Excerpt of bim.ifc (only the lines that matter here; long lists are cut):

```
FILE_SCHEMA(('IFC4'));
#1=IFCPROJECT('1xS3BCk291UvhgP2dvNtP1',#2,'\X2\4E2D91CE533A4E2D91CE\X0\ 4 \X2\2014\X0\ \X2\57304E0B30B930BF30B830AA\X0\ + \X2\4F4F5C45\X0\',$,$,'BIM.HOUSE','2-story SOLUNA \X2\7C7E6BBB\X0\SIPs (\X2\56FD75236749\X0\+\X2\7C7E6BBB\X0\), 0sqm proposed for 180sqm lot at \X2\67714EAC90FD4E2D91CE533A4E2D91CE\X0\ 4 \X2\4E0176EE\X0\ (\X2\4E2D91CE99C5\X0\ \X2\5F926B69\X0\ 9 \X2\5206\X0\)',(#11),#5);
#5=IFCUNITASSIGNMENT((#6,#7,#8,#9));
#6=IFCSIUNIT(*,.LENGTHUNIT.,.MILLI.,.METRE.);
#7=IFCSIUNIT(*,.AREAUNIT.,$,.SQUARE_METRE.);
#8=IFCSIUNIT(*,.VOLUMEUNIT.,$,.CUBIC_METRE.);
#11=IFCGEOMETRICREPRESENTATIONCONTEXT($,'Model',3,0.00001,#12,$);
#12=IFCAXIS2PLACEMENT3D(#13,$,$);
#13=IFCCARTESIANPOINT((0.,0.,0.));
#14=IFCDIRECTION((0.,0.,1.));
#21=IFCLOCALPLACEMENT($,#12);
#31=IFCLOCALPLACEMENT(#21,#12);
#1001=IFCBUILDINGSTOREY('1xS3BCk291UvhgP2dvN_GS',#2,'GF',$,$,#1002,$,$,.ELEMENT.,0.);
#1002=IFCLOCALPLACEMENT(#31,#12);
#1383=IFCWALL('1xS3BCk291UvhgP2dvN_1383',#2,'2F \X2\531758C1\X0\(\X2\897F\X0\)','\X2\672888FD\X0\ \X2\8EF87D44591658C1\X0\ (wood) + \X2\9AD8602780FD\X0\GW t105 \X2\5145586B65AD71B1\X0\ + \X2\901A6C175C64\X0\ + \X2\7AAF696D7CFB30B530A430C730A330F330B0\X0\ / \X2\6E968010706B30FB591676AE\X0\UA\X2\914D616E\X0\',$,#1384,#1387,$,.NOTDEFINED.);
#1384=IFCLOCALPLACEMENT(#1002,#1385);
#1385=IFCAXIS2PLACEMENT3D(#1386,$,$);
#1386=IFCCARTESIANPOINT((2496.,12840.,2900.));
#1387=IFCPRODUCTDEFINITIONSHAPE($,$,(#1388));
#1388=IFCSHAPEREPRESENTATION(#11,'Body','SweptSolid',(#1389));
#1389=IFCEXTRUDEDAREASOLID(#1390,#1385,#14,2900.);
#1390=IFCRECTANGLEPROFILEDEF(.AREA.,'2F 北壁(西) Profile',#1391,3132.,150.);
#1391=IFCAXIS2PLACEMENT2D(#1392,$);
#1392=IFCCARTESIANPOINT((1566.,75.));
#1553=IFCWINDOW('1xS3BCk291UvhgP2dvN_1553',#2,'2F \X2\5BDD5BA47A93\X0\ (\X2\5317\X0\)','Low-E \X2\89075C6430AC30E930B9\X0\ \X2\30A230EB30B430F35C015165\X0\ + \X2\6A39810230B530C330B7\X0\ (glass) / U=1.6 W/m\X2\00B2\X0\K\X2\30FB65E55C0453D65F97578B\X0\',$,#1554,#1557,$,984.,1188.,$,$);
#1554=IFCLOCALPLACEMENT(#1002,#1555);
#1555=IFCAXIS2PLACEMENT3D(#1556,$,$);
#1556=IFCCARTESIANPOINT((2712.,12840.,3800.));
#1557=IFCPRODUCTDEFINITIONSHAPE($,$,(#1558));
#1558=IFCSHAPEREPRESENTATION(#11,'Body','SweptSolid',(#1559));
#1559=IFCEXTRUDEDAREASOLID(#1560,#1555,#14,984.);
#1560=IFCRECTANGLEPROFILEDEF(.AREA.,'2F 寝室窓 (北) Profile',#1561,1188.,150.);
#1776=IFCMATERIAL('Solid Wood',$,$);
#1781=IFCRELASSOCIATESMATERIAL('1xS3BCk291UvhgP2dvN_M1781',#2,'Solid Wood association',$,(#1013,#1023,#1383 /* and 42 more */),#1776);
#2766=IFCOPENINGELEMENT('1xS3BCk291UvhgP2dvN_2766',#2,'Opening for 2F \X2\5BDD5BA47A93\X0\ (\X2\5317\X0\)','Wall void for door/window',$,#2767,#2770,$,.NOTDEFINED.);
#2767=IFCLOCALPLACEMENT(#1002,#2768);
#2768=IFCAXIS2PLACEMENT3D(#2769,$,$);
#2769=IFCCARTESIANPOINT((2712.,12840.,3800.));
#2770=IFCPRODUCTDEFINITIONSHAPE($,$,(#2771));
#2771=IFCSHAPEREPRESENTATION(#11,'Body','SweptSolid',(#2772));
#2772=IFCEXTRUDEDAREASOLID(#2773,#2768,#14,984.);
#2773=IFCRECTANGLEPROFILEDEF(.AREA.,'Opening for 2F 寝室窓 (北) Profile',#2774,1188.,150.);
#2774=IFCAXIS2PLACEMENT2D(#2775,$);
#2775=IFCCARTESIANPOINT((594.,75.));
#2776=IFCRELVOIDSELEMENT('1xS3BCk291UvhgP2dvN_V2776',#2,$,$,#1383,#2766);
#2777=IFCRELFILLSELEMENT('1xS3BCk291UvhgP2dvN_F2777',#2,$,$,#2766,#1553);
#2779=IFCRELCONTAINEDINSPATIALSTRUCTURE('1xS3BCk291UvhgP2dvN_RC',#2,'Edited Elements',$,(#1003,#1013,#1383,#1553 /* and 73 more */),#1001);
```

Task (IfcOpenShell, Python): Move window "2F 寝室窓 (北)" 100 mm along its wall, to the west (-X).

```python
import ifcopenshell
import ifcopenshell.api.geometry
import ifcopenshell.util.placement
import ifcopenshell.util.unit

model = ifcopenshell.open("bim.ifc")
unit_scale = ifcopenshell.util.unit.calculate_unit_scale(model)

window = model.by_id(1553)
opening = window.FillsVoids[0].RelatingOpeningElement
wall = opening.VoidsElements[0].RelatingBuildingElement

wall_matrix = ifcopenshell.util.placement.get_local_placement(wall.ObjectPlacement)
shift = wall_matrix[:3, 0] * -0.1 / unit_scale
before = ifcopenshell.util.placement.get_local_placement(window.ObjectPlacement)[:3, 3].copy()

# The window is not placed relative to its opening, so move both.
for product in (opening, window):
    matrix = ifcopenshell.util.placement.get_local_placement(product.ObjectPlacement)
    matrix[:3, 3] += shift
    ifcopenshell.api.geometry.edit_object_placement(model, product=product, matrix=matrix, is_si=False)

after = ifcopenshell.util.placement.get_local_placement(window.ObjectPlacement)[:3, 3]
print("window moved by", (after - before).round(3) + 0.0)

model.write("bim_edited.ifc")
```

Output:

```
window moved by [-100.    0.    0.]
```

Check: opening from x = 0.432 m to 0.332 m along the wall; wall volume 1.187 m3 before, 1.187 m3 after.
